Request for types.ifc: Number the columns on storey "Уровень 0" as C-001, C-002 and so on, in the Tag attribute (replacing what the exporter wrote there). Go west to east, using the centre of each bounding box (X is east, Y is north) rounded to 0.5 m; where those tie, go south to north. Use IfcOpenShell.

First a look at what the model holds.

```python
import ifcopenshell
import ifcopenshell.util.element
import ifcopenshell.util.placement

model = ifcopenshell.open("types.ifc")
print(model.schema)
storey = next(s for s in model.by_type("IfcBuildingStorey") if s.Name == "Уровень 0")
columns = [e for e in ifcopenshell.util.element.get_decomposition(storey) if e.is_a("IfcColumn")]
for e in sorted(columns, key=lambda e: e.id()):
    origin = ifcopenshell.util.placement.get_local_placement(e.ObjectPlacement)[:3, 3]
    print(e.id(), e.Tag, e.Name, origin.round(2) + 0.0, sep=" | ")
```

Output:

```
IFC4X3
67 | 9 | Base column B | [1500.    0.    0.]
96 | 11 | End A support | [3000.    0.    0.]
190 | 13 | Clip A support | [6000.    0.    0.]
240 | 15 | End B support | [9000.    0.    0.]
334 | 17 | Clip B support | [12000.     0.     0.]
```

```python
import ifcopenshell
import ifcopenshell.geom
import ifcopenshell.util.element
import ifcopenshell.util.shape

model = ifcopenshell.open("types.ifc")
settings = ifcopenshell.geom.settings()
settings.set("use-world-coords", True)


def centre(element):
    shape = ifcopenshell.geom.create_shape(settings, element)
    return ifcopenshell.util.shape.get_bbox_centroid(shape.geometry)


storey = next(s for s in model.by_type("IfcBuildingStorey") if s.Name == "Уровень 0")
columns = [e for e in ifcopenshell.util.element.get_decomposition(storey) if e.is_a("IfcColumn")]

# Insertion points can sit at a corner or the storey origin, so sort by the geometry (in metres).
centres = {e: centre(e) for e in columns}
columns.sort(key=lambda e: (round(centres[e][0] / 0.5), centres[e][1]))

for i, e in enumerate(columns, start=1):
    number = f"C-0{i:02d}"
    e.Tag = number
    print(e.id(), number)

model.write("types_updated.ifc")
```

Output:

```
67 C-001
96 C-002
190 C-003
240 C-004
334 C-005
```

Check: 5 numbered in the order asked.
